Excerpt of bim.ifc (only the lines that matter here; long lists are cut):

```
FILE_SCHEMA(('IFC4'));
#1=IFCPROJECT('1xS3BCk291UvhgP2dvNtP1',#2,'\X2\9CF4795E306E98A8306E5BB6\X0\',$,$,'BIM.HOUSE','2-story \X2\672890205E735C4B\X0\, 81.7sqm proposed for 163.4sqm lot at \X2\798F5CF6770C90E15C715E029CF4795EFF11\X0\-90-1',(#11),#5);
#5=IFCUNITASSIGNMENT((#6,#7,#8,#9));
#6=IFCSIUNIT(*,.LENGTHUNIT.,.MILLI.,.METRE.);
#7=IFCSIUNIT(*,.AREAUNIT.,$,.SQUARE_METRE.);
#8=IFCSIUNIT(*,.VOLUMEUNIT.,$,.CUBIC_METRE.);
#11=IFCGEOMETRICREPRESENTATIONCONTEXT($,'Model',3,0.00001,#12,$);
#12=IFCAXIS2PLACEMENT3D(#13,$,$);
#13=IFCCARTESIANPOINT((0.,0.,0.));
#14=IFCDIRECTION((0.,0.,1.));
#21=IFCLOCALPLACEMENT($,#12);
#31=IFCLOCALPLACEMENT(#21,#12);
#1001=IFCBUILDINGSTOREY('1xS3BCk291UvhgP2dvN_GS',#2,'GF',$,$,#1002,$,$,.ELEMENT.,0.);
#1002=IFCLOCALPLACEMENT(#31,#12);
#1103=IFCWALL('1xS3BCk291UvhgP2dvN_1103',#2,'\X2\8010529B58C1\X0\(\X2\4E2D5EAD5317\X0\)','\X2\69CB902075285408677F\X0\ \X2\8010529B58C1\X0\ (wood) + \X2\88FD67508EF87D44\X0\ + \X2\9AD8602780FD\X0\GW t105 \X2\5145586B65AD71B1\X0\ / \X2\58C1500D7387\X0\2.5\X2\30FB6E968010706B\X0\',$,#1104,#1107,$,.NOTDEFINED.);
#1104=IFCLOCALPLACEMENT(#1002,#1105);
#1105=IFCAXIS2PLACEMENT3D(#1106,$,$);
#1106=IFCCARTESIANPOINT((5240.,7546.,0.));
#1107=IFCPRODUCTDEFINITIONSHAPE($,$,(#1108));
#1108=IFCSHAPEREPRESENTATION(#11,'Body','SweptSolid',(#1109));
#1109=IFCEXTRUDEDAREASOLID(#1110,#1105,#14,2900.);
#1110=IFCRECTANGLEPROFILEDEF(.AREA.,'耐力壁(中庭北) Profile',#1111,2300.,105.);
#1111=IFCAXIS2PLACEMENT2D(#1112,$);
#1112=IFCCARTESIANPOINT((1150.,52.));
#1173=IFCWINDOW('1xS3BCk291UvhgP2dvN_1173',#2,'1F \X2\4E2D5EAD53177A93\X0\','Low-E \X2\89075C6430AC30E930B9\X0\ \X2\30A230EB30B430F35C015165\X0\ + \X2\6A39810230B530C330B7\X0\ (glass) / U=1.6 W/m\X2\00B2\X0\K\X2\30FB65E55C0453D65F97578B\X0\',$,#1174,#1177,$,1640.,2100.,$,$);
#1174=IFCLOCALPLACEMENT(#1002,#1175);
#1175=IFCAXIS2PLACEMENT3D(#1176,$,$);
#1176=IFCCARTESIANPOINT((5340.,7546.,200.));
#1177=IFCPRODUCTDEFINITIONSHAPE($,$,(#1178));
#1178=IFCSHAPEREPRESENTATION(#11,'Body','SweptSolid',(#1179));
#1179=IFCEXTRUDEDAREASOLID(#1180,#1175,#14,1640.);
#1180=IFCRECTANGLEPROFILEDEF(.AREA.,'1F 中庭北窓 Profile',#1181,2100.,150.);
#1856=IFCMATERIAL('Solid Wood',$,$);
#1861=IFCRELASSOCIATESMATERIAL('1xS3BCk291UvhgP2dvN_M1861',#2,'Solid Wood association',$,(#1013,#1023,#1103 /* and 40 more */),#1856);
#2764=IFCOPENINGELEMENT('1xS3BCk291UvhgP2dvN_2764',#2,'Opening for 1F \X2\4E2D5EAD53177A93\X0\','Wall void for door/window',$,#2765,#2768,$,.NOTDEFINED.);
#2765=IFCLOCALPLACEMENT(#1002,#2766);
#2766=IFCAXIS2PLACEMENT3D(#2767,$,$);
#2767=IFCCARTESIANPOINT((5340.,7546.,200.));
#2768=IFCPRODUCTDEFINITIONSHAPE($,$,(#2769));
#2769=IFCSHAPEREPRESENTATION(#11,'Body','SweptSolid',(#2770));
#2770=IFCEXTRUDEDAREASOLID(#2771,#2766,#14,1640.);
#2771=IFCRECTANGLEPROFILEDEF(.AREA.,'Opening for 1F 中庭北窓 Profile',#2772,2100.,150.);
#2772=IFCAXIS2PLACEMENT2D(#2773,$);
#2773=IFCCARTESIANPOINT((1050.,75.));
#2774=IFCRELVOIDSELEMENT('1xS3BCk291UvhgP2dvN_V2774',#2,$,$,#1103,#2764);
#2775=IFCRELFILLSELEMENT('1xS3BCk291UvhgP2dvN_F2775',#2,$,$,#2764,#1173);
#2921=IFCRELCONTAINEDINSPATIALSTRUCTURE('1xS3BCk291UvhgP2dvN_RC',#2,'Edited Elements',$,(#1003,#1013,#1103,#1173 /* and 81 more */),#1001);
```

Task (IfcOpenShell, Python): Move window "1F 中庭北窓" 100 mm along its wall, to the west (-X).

```python
import ifcopenshell
import ifcopenshell.api.geometry
import ifcopenshell.util.placement
import ifcopenshell.util.unit

model = ifcopenshell.open("bim.ifc")
unit_scale = ifcopenshell.util.unit.calculate_unit_scale(model)

window = model.by_guid("1xS3BCk291UvhgP2dvN_1173")
opening = window.FillsVoids[0].RelatingOpeningElement
wall = opening.VoidsElements[0].RelatingBuildingElement

wall_matrix = ifcopenshell.util.placement.get_local_placement(wall.ObjectPlacement)
shift = wall_matrix[:3, 0] * -0.1 / unit_scale
before = ifcopenshell.util.placement.get_local_placement(window.ObjectPlacement)[:3, 3].copy()

# The window is not placed relative to its opening, so move both.
for product in (opening, window):
    matrix = ifcopenshell.util.placement.get_local_placement(product.ObjectPlacement)
    matrix[:3, 3] += shift
    ifcopenshell.api.geometry.edit_object_placement(model, product=product, matrix=matrix, is_si=False)

after = ifcopenshell.util.placement.get_local_placement(window.ObjectPlacement)[:3, 3]
print("window moved by", (after - before).round(3) + 0.0)

model.write("bim_updated.ifc")
```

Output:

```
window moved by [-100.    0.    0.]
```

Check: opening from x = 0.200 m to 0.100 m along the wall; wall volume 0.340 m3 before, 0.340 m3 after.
